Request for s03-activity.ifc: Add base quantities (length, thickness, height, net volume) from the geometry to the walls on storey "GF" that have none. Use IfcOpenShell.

First a look at what the model holds.

```python
import ifcopenshell
import ifcopenshell.util.element
import ifcopenshell.util.unit

model = ifcopenshell.open("s03-activity.ifc")
print(model.schema)
for unit_type in ("LENGTHUNIT", "AREAUNIT", "VOLUMEUNIT"):
    print(unit_type, ifcopenshell.util.unit.calculate_unit_scale(model, unit_type))
storey = next(s for s in model.by_type("IfcBuildingStorey") if s.Name == "GF")
walls = [e for e in ifcopenshell.util.element.get_decomposition(storey) if e.is_a("IfcWall")]
for e in sorted(walls, key=lambda e: e.id()):
    print(e.id(), e.is_a(), e.Name, list(ifcopenshell.util.element.get_psets(e, qtos_only=True)), sep=" | ")
```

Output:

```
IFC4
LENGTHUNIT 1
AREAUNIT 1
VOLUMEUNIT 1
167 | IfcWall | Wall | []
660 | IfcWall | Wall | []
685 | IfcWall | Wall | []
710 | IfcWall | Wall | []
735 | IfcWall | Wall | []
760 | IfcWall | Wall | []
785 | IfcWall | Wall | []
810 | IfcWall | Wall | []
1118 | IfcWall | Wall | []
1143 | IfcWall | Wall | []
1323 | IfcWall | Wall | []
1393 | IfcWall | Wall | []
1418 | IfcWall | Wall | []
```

```python
import ifcopenshell
import ifcopenshell.api.pset
import ifcopenshell.geom
import ifcopenshell.util.element
import ifcopenshell.util.shape
import ifcopenshell.util.unit

model = ifcopenshell.open("s03-activity.ifc")
unit_scale = ifcopenshell.util.unit.calculate_unit_scale(model)
volume_scale = ifcopenshell.util.unit.calculate_unit_scale(model, "VOLUMEUNIT")
settings = ifcopenshell.geom.settings()

storey = next(s for s in model.by_type("IfcBuildingStorey") if s.Name == "GF")
walls = [e for e in ifcopenshell.util.element.get_decomposition(storey) if e.is_a("IfcWall")]

for e in sorted(walls, key=lambda e: e.id()):
    if ifcopenshell.util.element.get_psets(e, qtos_only=True, should_inherit=False):
        continue
    # Geometry comes back in metres, in the element's own axes.
    shape = ifcopenshell.geom.create_shape(settings, e)
    values = {
        "Length": ifcopenshell.util.shape.get_x(shape.geometry) / unit_scale,
        "Width": ifcopenshell.util.shape.get_y(shape.geometry) / unit_scale,
        "Height": ifcopenshell.util.shape.get_z(shape.geometry) / unit_scale,
        "NetVolume": ifcopenshell.util.shape.get_volume(shape.geometry) / volume_scale,
    }
    qto = ifcopenshell.api.pset.add_qto(model, product=e, name="Qto_WallBaseQuantities")
    ifcopenshell.api.pset.edit_qto(model, qto=qto, properties=values)
    print(e.id(), {k: round(v, 3) for k, v in values.items()})

model.write("s03-activity_rev.ifc")
```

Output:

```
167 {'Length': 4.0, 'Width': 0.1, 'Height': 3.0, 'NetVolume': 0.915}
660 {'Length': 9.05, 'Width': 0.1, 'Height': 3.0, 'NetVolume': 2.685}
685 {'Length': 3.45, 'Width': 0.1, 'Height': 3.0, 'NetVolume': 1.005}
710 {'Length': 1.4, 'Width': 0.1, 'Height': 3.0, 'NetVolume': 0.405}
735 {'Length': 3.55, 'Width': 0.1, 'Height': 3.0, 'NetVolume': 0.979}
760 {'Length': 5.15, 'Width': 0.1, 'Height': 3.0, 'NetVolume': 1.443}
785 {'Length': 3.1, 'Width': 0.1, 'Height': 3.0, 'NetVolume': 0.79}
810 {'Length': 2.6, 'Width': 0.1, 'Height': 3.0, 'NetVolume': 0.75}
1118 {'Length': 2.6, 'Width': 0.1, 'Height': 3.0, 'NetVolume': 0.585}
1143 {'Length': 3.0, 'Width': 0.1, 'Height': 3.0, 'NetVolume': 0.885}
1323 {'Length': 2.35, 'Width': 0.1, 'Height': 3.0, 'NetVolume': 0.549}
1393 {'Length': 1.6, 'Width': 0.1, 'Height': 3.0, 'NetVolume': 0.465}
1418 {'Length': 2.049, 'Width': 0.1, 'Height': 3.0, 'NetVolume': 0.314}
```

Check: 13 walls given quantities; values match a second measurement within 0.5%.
